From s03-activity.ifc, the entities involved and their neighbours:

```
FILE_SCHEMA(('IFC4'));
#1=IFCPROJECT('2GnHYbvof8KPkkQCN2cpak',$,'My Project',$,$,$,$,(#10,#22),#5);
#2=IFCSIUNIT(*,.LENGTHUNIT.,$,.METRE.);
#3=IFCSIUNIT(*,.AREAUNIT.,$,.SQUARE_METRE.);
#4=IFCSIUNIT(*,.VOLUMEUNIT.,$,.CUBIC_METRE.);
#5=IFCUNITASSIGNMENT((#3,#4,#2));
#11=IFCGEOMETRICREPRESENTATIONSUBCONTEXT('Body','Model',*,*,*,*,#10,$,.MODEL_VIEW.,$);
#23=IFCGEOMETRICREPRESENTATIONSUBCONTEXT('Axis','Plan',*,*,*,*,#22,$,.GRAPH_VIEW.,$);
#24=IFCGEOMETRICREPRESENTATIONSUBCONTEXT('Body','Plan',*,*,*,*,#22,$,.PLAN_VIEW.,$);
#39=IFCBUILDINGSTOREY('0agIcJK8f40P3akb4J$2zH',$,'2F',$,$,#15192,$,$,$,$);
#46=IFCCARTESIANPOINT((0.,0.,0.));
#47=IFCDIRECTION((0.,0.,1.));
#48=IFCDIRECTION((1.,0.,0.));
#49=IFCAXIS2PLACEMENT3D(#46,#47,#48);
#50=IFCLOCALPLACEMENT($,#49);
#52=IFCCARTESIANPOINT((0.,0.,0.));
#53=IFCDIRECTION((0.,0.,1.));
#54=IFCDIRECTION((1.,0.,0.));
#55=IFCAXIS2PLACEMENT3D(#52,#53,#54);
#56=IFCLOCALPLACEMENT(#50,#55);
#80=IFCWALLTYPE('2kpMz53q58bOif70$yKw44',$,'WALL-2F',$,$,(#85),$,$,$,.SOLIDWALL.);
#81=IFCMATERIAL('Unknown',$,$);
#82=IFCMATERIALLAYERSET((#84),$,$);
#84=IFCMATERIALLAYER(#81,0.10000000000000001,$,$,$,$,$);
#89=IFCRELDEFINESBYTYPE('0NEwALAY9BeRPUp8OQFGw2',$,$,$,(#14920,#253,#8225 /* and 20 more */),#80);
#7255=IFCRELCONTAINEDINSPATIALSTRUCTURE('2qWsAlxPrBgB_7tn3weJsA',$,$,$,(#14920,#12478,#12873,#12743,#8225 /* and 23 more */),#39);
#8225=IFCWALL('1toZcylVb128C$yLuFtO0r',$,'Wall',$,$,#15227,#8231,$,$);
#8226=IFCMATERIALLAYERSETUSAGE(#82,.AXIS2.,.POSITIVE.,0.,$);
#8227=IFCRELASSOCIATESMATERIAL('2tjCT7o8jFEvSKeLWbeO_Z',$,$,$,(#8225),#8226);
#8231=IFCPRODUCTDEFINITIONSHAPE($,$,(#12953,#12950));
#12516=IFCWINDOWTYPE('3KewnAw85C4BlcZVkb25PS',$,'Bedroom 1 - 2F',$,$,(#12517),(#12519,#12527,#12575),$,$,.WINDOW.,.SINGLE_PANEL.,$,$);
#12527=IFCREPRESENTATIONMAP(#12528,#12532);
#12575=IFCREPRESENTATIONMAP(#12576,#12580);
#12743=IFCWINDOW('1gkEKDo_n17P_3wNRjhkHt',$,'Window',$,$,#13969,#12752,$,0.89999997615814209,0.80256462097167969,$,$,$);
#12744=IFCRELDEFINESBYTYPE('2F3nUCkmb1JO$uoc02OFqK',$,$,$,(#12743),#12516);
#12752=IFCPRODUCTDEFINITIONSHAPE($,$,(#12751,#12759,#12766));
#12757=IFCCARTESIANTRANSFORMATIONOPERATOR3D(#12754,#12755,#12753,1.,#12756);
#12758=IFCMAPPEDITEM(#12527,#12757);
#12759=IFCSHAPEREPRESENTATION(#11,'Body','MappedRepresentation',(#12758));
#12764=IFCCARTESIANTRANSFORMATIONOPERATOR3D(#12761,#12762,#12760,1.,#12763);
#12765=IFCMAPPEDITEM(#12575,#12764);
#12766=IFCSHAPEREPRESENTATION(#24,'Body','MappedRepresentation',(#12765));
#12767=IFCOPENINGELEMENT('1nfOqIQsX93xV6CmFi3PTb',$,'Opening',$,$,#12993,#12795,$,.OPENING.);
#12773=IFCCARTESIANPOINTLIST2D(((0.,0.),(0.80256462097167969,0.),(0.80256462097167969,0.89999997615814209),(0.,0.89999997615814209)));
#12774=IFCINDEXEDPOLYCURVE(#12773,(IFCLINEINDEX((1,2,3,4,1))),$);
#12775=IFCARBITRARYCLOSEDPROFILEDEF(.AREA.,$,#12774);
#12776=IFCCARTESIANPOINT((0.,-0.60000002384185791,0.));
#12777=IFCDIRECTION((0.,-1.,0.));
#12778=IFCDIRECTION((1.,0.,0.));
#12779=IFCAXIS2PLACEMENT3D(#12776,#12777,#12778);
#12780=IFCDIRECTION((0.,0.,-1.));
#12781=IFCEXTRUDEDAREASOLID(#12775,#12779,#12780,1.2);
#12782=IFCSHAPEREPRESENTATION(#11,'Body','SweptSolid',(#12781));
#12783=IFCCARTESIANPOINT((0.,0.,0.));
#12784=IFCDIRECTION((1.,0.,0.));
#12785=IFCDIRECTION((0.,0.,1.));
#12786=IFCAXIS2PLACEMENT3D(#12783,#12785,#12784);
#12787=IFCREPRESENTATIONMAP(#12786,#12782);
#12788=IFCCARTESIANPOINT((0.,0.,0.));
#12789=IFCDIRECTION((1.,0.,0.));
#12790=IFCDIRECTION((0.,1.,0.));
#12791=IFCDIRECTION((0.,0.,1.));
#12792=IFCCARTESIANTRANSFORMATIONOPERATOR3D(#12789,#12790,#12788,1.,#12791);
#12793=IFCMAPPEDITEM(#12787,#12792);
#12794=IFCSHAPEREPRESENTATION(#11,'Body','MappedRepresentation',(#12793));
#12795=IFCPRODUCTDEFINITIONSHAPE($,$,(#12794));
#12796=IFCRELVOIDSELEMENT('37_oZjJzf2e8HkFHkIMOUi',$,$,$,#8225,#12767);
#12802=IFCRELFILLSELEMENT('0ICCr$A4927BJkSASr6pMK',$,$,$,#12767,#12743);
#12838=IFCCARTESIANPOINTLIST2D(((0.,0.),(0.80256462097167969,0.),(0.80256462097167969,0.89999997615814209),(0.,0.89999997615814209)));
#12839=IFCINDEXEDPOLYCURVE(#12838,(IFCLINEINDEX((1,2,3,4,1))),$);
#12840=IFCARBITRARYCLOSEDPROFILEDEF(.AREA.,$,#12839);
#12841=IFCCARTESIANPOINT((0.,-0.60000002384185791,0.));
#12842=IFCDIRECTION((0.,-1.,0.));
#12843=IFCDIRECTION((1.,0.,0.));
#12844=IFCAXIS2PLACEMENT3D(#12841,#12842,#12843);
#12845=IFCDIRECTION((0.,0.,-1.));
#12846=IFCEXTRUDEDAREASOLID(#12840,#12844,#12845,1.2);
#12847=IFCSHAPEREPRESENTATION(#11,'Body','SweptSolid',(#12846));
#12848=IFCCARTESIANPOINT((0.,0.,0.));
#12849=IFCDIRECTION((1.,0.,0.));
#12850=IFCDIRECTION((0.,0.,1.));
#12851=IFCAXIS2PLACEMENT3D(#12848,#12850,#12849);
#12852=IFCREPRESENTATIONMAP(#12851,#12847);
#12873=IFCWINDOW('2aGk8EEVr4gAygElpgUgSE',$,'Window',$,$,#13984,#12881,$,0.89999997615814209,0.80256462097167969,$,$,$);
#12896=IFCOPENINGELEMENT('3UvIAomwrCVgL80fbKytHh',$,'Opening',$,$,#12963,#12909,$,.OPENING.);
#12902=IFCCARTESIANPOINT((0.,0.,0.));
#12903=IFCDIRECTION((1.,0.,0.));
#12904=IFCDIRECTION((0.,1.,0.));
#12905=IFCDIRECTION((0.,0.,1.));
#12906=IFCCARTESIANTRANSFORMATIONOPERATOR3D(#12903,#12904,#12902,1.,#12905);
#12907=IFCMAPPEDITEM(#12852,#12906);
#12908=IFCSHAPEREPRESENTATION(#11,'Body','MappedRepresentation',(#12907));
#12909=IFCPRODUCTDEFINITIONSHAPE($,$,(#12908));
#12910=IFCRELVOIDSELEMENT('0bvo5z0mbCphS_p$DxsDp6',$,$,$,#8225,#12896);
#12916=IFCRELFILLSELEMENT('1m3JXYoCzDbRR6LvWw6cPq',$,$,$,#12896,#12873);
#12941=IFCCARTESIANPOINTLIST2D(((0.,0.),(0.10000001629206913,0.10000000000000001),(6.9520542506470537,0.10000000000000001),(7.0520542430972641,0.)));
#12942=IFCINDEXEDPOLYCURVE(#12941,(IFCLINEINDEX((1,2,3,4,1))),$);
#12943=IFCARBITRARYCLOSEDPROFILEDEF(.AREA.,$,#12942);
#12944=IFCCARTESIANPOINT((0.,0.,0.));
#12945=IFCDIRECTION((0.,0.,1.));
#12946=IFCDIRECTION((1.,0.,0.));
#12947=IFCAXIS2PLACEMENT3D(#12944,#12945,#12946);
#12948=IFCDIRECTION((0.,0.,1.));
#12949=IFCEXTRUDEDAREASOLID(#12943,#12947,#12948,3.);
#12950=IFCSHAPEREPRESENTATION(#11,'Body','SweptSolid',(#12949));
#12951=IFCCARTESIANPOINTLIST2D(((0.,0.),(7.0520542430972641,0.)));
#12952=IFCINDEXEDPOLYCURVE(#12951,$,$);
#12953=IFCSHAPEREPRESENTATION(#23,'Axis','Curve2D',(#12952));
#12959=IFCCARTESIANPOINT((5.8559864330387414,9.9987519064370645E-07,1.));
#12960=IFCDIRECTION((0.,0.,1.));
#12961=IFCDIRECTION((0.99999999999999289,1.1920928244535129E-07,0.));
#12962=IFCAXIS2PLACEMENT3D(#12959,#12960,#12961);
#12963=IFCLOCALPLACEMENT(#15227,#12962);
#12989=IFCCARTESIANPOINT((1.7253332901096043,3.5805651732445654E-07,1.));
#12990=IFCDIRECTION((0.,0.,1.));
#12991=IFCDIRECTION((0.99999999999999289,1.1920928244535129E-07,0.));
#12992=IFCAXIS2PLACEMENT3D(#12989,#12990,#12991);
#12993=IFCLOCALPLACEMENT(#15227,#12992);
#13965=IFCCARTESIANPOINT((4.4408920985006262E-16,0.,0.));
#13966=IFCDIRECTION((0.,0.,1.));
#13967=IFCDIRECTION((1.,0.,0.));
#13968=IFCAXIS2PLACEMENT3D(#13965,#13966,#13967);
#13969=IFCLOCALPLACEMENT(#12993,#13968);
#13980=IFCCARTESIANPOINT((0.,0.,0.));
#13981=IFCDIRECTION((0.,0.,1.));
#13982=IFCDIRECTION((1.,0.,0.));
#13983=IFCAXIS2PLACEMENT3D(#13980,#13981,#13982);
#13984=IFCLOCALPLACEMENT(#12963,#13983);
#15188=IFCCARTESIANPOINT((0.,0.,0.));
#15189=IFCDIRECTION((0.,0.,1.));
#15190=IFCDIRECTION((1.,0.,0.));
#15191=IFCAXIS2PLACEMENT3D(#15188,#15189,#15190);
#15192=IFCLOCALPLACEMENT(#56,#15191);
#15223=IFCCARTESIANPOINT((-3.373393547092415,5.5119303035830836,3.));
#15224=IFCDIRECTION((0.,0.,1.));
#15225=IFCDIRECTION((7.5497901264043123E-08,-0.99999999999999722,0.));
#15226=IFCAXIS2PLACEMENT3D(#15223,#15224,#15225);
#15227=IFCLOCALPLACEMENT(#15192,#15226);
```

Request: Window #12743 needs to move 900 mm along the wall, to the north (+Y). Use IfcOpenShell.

```python
import ifcopenshell
import ifcopenshell.api.geometry
import ifcopenshell.util.placement

model = ifcopenshell.open("s03-activity.ifc")

window = model.by_id(12743)
opening = window.FillsVoids[0].RelatingOpeningElement
wall = opening.VoidsElements[0].RelatingBuildingElement

wall_matrix = ifcopenshell.util.placement.get_local_placement(wall.ObjectPlacement)
shift = wall_matrix[:3, 0] * -0.9
before = ifcopenshell.util.placement.get_local_placement(window.ObjectPlacement)[:3, 3].copy()

# The window is placed relative to its opening, so it follows when the opening moves.
matrix = ifcopenshell.util.placement.get_local_placement(opening.ObjectPlacement)
matrix[:3, 3] += shift
ifcopenshell.api.geometry.edit_object_placement(
    model, product=opening, matrix=matrix, is_si=False, should_transform_children=True
)

after = ifcopenshell.util.placement.get_local_placement(window.ObjectPlacement)[:3, 3]
print("window moved by", (after - before).round(3) + 0.0)

model.write("s03-activity-out.ifc")
```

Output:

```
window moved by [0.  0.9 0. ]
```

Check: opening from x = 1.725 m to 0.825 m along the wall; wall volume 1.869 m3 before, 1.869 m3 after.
